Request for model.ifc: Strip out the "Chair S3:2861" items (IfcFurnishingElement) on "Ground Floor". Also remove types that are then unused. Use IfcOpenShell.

First a look at what the model holds.

```python
import ifcopenshell
import ifcopenshell.util.element

model = ifcopenshell.open("model.ifc")
print(model.schema)
storey = next(s for s in model.by_type("IfcBuildingStorey") if s.Name == "Ground Floor")
furniture = [e for e in ifcopenshell.util.element.get_decomposition(storey) if e.is_a("IfcFurnishingElement")]
seen = {}
for e in furniture:
    element_type = ifcopenshell.util.element.get_type(e)
    name = element_type.Name if element_type not in (None, e) else None
    seen[name] = seen.get(name, 0) + 1
for name, count in sorted(seen.items(), key=str):
    print(count, "x", name)
```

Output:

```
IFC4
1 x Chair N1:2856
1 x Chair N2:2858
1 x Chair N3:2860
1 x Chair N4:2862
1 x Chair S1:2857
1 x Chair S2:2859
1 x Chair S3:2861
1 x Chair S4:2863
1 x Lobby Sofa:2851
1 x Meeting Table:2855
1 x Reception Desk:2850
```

```python
import ifcopenshell
import ifcopenshell.api.root
import ifcopenshell.util.element

model = ifcopenshell.open("model.ifc")

storey = next(s for s in model.by_type("IfcBuildingStorey") if s.Name == "Ground Floor")
furniture = [e for e in ifcopenshell.util.element.get_decomposition(storey) if e.is_a("IfcFurnishingElement")]
targets = [e for e in furniture if (t := ifcopenshell.util.element.get_type(e)) not in (None, e) and t.Name == "Chair S3:2861"]
types = {ifcopenshell.util.element.get_type(e) for e in targets} - {None, *targets}

for e in targets:
    ifcopenshell.api.root.remove_product(model, product=e)
print(len(targets), "removed")

unused = [t for t in types if not ifcopenshell.util.element.get_types(t)]
for t in unused:
    ifcopenshell.api.root.remove_product(model, product=t)
print(len(unused), "unused types removed")

model.write("model_updated.ifc")
```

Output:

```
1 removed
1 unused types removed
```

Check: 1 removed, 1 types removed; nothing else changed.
